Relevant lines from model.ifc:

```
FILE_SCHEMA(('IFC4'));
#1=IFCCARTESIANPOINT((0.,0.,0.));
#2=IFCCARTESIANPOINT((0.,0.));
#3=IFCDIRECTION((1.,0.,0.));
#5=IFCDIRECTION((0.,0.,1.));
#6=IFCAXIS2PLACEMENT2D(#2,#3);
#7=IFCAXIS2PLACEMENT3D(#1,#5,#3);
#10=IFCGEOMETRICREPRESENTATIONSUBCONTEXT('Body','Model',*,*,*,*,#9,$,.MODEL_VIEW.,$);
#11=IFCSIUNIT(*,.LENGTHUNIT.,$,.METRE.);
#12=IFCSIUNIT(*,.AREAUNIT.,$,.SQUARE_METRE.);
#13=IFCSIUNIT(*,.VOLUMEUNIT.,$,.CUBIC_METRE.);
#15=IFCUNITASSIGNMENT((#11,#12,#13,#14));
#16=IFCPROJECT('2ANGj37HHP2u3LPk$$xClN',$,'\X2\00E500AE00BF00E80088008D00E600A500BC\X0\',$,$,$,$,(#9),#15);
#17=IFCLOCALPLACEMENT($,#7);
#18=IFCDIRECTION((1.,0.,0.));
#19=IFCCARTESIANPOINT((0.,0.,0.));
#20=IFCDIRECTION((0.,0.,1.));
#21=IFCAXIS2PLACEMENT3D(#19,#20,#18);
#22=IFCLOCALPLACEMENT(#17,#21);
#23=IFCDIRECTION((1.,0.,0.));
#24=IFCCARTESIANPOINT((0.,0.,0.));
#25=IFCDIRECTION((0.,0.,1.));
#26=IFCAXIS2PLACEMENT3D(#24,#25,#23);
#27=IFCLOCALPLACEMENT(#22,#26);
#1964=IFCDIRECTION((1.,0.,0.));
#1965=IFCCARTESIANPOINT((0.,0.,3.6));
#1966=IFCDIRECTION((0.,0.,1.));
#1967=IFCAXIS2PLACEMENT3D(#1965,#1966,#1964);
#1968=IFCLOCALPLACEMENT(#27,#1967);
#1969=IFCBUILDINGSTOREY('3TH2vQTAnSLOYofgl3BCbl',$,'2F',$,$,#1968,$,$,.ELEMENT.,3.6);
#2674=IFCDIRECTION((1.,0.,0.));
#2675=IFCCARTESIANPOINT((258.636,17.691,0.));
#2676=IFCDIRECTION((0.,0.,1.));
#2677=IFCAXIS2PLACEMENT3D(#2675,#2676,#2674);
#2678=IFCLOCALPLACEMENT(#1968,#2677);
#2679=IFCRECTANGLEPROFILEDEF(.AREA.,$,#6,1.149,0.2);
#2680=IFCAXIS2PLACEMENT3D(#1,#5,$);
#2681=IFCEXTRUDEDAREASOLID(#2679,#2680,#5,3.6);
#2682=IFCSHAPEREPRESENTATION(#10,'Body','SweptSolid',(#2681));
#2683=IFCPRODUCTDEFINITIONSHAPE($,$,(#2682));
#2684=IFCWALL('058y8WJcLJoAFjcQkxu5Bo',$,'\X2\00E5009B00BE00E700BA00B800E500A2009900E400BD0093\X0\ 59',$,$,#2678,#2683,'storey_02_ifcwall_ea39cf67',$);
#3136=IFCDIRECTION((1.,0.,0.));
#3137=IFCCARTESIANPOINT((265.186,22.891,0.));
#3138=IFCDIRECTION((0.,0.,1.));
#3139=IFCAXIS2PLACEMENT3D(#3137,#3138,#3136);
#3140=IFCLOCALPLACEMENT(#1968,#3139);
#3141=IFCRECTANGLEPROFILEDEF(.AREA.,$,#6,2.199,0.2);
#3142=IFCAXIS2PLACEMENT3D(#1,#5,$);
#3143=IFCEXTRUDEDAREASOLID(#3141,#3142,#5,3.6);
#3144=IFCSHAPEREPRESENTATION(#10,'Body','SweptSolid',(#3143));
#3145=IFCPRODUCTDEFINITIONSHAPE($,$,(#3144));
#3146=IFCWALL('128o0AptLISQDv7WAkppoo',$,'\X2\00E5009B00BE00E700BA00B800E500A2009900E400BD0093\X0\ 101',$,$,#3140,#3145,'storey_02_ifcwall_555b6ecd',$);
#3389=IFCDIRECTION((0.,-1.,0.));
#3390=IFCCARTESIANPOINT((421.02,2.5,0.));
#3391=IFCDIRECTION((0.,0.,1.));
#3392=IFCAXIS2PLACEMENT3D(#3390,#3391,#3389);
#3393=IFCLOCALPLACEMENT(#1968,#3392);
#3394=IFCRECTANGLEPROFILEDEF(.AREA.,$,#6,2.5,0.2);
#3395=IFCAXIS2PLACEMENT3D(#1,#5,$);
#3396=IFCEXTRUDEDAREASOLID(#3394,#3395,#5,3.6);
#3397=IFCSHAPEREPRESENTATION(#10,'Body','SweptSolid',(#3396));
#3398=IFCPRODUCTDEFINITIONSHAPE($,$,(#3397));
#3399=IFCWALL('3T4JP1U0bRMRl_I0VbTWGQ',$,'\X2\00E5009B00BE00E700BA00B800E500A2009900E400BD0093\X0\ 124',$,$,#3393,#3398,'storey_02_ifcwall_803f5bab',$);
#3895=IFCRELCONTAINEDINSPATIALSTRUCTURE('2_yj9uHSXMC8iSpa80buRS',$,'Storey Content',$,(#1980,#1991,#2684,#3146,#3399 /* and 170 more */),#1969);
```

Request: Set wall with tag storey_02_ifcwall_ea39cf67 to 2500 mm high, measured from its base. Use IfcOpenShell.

```python
import ifcopenshell
import ifcopenshell.geom
import ifcopenshell.util.representation
import ifcopenshell.util.shape

model = ifcopenshell.open("model.ifc")
settings = ifcopenshell.geom.settings()


def volume(element):
    """Net volume in cubic metres, openings subtracted."""
    shape = ifcopenshell.geom.create_shape(settings, element)
    return ifcopenshell.util.shape.get_volume(shape.geometry)


wall = model.by_id(2684)
before = volume(wall)

body = ifcopenshell.util.representation.get_representation(wall, "Model", "Body")
solid = body.Items[0]
old_height = solid.Depth
solid.Depth = 2.5
after = volume(wall)

print(f"height {old_height:g} -> {solid.Depth:g}, volume {before:.3f} -> {after:.3f} m3")

model.write("model_edited.ifc")
```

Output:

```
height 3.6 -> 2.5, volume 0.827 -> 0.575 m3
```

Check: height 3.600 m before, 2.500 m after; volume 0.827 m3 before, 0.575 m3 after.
